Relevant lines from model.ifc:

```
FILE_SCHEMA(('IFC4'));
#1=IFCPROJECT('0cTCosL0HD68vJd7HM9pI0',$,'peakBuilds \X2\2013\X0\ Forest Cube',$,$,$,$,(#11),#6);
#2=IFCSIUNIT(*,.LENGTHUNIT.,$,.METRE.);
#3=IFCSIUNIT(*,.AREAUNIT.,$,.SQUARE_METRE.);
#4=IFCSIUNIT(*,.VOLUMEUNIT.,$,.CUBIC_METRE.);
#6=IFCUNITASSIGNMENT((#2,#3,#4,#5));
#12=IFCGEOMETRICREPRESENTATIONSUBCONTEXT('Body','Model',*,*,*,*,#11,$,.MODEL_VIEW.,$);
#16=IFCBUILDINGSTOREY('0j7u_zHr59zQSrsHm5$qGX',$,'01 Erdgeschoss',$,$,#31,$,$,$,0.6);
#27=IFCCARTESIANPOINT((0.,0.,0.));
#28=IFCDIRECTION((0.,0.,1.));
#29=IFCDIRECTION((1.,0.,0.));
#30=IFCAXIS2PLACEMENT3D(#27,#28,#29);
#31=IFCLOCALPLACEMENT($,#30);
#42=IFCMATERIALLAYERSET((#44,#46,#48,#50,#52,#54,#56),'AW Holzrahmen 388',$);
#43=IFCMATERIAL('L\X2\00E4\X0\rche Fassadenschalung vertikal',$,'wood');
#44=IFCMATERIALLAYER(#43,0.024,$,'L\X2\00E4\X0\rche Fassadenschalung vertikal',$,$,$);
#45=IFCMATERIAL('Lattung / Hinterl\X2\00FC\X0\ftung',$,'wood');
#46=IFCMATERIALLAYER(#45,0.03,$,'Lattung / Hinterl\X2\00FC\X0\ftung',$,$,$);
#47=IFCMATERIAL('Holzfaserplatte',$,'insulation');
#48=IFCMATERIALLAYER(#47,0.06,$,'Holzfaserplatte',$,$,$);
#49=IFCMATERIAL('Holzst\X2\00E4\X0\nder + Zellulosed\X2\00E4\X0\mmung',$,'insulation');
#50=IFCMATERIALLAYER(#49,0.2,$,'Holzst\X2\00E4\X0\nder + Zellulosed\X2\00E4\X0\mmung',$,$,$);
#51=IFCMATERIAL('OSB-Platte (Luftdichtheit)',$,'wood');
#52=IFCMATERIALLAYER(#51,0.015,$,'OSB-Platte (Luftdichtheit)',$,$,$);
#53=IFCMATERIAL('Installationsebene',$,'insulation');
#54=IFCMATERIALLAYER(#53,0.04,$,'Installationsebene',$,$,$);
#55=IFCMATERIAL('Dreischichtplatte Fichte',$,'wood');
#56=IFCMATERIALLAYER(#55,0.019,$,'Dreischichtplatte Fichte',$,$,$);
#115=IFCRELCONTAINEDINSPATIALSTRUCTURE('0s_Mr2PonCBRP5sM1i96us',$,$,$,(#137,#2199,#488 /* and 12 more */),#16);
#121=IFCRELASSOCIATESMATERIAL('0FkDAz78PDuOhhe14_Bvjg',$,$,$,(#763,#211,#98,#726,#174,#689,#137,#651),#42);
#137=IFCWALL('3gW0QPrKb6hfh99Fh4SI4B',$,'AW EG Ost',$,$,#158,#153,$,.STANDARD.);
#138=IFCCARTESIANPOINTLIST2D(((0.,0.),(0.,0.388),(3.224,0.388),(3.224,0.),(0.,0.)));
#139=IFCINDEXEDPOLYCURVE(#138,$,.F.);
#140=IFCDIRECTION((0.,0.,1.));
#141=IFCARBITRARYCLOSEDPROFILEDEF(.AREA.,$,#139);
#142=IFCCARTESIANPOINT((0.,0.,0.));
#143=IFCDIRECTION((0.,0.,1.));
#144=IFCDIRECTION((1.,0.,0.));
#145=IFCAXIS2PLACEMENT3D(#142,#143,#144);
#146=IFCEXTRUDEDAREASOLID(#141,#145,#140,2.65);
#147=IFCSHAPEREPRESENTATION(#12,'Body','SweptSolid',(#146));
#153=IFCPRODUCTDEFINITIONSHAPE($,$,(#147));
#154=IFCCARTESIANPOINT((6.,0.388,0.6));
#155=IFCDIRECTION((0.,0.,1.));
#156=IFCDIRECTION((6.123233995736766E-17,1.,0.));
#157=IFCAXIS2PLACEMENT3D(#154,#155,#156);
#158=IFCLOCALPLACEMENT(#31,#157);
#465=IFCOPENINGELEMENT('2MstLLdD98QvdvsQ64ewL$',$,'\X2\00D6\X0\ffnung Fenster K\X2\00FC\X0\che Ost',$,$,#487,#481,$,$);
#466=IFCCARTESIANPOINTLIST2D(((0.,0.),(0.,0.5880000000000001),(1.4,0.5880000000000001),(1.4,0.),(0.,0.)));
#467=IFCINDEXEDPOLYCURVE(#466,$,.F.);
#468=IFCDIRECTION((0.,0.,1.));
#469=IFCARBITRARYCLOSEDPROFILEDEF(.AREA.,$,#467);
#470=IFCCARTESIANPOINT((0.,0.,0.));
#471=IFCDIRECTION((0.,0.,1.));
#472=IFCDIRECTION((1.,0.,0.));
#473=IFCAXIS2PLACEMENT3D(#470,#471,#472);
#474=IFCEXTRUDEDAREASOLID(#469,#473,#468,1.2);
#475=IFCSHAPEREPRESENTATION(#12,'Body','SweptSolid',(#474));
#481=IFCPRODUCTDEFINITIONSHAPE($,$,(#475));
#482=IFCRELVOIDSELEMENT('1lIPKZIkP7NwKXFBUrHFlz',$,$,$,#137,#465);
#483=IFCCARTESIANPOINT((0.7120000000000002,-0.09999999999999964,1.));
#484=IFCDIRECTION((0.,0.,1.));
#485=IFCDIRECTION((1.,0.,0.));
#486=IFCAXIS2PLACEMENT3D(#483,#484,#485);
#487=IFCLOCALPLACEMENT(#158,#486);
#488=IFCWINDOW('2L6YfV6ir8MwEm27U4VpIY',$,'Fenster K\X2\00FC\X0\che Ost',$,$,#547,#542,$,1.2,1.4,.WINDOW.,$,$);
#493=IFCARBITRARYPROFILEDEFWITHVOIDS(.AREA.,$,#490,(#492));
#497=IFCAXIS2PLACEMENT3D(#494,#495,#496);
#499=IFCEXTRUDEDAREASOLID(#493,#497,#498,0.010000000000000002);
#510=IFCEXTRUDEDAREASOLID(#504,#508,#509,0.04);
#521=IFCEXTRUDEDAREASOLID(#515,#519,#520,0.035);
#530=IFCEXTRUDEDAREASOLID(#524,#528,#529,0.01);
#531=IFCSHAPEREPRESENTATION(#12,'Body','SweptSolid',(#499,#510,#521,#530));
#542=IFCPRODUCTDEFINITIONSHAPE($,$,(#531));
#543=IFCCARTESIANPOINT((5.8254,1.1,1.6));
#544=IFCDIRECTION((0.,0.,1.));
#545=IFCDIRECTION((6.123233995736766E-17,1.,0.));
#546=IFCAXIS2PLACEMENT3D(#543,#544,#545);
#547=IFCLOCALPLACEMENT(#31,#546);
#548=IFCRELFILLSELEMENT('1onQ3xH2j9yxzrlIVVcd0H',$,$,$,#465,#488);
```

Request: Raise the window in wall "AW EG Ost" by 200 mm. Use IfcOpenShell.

```python
import numpy as np
import ifcopenshell
import ifcopenshell.api.geometry
import ifcopenshell.util.placement
import ifcopenshell.util.unit

model = ifcopenshell.open("model.ifc")
unit_scale = ifcopenshell.util.unit.calculate_unit_scale(model)

window = model.by_guid("2L6YfV6ir8MwEm27U4VpIY")
opening = window.FillsVoids[0].RelatingOpeningElement
dz = 0.2 / unit_scale

shift = np.array([0.0, 0.0, dz])
# The window is not placed relative to its opening, so move both.
for product in (opening, window):
    matrix = ifcopenshell.util.placement.get_local_placement(product.ObjectPlacement)
    matrix[:3, 3] += shift
    ifcopenshell.api.geometry.edit_object_placement(model, product=product, matrix=matrix, is_si=False)

print(f"moved by {dz * unit_scale:+.3f} m")

model.write("model_edited.ifc")
```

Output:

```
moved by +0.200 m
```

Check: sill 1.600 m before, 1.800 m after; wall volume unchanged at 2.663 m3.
